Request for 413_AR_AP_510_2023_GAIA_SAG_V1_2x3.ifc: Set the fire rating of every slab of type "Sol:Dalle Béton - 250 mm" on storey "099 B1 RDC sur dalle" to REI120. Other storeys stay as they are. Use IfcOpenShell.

First a look at what the model holds.

```python
import ifcopenshell
import ifcopenshell.util.element

model = ifcopenshell.open("413_AR_AP_510_2023_GAIA_SAG_V1_2x3.ifc")
print(model.schema)
storey = next(s for s in model.by_type("IfcBuildingStorey") if s.Name == "099 B1 RDC sur dalle")
slabs = [e for e in ifcopenshell.util.element.get_decomposition(storey) if e.is_a("IfcSlab")]
seen = {}
for e in slabs:
    element_type = ifcopenshell.util.element.get_type(e)
    key = (element_type.Name if element_type != e and element_type else None, ifcopenshell.util.element.get_pset(e, "Pset_SlabCommon", "FireRating"))
    seen[key] = seen.get(key, 0) + 1
for (name, value), count in sorted(seen.items(), key=str):
    print(count, "x", name, "|", value)
```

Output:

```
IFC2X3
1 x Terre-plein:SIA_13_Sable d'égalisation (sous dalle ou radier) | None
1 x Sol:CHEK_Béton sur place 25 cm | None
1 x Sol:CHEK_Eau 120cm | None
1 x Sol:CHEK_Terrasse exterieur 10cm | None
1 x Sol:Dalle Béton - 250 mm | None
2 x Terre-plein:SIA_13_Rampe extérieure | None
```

```python
import ifcopenshell
import ifcopenshell.api.pset
import ifcopenshell.util.element

model = ifcopenshell.open("413_AR_AP_510_2023_GAIA_SAG_V1_2x3.ifc")

storey = next(s for s in model.by_type("IfcBuildingStorey") if s.Name == "099 B1 RDC sur dalle")
slabs = [e for e in ifcopenshell.util.element.get_decomposition(storey) if e.is_a("IfcSlab")]

count = 0
for e in slabs:
    element_type = ifcopenshell.util.element.get_type(e)
    if element_type in (None, e) or element_type.Name != "Sol:Dalle Béton - 250 mm":
        continue
    # add_pset returns the element's existing set when there is one.
    pset = ifcopenshell.api.pset.add_pset(model, product=e, name="Pset_SlabCommon")
    ifcopenshell.api.pset.edit_pset(model, pset=pset, properties={"FireRating": "REI120"})
    count += 1

print(count, "slabs updated")

model.write("413_AR_AP_510_2023_GAIA_SAG_V1_2x3_updated.ifc")
```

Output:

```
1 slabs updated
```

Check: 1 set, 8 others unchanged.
